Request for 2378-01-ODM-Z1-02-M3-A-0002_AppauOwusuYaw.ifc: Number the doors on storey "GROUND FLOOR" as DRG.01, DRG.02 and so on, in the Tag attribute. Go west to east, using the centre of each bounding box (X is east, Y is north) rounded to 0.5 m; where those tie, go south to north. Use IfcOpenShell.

First a look at what the model holds.

```python
import ifcopenshell
import ifcopenshell.util.element
import ifcopenshell.util.placement

model = ifcopenshell.open("2378-01-ODM-Z1-02-M3-A-0002_AppauOwusuYaw.ifc")
print(model.schema)
storey = next(s for s in model.by_type("IfcBuildingStorey") if s.Name == "GROUND FLOOR")
doors = [e for e in ifcopenshell.util.element.get_decomposition(storey) if e.is_a("IfcDoor")]
for e in sorted(doors, key=lambda e: e.id()):
    origin = ifcopenshell.util.placement.get_local_placement(e.ObjectPlacement)[:3, 3]
    print(e.id(), e.Tag, e.Name, origin.round(2) + 0.0, sep=" | ")
```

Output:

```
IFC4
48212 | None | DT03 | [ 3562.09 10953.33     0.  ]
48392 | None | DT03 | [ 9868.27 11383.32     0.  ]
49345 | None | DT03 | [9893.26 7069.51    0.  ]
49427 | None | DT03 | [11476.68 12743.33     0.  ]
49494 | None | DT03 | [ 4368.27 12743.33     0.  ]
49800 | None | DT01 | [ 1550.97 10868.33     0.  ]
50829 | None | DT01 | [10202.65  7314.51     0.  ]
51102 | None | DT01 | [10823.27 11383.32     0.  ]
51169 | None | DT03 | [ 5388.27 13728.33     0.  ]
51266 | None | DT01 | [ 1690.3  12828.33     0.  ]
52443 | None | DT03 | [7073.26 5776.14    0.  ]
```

```python
import ifcopenshell
import ifcopenshell.geom
import ifcopenshell.util.element
import ifcopenshell.util.shape

model = ifcopenshell.open("2378-01-ODM-Z1-02-M3-A-0002_AppauOwusuYaw.ifc")
settings = ifcopenshell.geom.settings()
settings.set("use-world-coords", True)


def centre(element):
    shape = ifcopenshell.geom.create_shape(settings, element)
    return ifcopenshell.util.shape.get_bbox_centroid(shape.geometry)


storey = next(s for s in model.by_type("IfcBuildingStorey") if s.Name == "GROUND FLOOR")
doors = [e for e in ifcopenshell.util.element.get_decomposition(storey) if e.is_a("IfcDoor")]

# Insertion points can sit at a corner or the storey origin, so sort by the geometry (in metres).
centres = {e: centre(e) for e in doors}
doors.sort(key=lambda e: (round(centres[e][0] / 0.5), centres[e][1]))

for i, e in enumerate(doors, start=1):
    number = f"DRG.{i:02d}"
    e.Tag = number
    print(e.id(), number)

model.write("2378-01-ODM-Z1-02-M3-A-0002_AppauOwusuYaw_rev.ifc")
```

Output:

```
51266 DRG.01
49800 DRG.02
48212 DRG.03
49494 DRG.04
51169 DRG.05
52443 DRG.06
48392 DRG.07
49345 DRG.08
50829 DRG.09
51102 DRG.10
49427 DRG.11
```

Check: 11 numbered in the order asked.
